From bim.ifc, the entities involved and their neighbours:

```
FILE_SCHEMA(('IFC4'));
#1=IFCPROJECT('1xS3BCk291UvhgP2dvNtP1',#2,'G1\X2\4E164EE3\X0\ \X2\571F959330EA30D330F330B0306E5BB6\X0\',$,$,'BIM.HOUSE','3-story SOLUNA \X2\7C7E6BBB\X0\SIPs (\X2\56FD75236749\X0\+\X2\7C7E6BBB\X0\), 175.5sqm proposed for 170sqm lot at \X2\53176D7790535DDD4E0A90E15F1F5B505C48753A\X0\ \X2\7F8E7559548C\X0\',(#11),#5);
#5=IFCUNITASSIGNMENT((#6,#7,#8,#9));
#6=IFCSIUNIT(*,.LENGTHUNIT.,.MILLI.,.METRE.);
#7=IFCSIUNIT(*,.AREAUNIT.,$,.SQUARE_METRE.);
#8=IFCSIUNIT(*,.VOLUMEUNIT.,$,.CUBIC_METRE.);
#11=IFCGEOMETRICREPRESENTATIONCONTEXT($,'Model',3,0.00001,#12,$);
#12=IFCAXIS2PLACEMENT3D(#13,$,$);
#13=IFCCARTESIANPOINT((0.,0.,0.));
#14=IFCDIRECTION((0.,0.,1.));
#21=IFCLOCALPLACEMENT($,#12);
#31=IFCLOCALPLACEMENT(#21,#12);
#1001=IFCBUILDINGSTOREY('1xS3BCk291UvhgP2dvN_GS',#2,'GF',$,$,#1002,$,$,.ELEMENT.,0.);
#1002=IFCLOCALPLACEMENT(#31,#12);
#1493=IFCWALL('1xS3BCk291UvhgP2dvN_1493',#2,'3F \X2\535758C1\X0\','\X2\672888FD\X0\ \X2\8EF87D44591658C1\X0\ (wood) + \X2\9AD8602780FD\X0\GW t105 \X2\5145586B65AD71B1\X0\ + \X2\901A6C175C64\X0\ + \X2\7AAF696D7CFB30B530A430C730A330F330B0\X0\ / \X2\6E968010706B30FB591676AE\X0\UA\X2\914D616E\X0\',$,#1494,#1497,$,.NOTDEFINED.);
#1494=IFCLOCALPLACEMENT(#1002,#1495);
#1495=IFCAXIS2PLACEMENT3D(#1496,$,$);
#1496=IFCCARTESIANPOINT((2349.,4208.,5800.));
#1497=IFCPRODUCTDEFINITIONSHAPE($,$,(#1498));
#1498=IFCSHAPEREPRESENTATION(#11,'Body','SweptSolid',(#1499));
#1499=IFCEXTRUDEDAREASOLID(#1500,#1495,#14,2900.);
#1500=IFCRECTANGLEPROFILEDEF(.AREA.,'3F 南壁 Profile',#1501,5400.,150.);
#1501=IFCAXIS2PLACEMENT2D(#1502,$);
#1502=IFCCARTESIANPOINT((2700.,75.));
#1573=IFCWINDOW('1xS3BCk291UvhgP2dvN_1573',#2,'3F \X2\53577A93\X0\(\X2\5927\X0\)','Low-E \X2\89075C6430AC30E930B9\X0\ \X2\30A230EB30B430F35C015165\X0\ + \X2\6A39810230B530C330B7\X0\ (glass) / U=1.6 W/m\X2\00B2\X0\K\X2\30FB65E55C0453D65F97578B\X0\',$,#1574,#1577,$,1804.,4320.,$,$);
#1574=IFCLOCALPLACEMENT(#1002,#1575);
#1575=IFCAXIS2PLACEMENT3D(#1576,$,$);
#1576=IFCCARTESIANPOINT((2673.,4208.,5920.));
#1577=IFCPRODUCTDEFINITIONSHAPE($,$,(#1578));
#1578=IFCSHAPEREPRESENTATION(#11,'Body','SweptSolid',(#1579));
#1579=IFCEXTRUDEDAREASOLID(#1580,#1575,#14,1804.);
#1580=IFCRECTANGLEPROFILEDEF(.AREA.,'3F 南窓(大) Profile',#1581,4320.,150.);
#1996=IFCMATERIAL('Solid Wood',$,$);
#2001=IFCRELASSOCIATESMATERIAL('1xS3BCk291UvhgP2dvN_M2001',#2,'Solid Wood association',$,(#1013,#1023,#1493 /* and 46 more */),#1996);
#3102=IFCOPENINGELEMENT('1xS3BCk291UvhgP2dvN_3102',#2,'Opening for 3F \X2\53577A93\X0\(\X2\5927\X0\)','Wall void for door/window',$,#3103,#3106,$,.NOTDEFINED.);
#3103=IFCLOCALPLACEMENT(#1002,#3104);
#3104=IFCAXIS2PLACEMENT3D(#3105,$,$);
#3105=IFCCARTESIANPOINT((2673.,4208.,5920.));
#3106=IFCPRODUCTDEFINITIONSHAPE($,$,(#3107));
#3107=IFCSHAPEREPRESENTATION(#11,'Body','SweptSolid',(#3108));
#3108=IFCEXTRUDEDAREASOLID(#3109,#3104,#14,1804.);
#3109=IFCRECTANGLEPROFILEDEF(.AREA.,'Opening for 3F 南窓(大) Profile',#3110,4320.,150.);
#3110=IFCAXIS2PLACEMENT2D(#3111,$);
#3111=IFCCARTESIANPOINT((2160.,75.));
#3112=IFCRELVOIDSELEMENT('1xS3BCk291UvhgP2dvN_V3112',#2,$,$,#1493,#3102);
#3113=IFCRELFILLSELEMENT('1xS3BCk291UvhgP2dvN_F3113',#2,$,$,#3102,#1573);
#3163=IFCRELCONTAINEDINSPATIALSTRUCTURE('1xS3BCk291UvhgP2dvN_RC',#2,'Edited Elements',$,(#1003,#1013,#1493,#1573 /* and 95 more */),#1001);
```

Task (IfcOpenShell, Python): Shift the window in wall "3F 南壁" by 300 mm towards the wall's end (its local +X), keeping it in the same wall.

```python
import ifcopenshell
import ifcopenshell.api.geometry
import ifcopenshell.util.placement
import ifcopenshell.util.unit

model = ifcopenshell.open("bim.ifc")
unit_scale = ifcopenshell.util.unit.calculate_unit_scale(model)

window = model.by_id(1573)
opening = window.FillsVoids[0].RelatingOpeningElement
wall = opening.VoidsElements[0].RelatingBuildingElement

wall_matrix = ifcopenshell.util.placement.get_local_placement(wall.ObjectPlacement)
shift = wall_matrix[:3, 0] * 0.3 / unit_scale
before = ifcopenshell.util.placement.get_local_placement(window.ObjectPlacement)[:3, 3].copy()

# The window is not placed relative to its opening, so move both.
for product in (opening, window):
    matrix = ifcopenshell.util.placement.get_local_placement(product.ObjectPlacement)
    matrix[:3, 3] += shift
    ifcopenshell.api.geometry.edit_object_placement(model, product=product, matrix=matrix, is_si=False)

after = ifcopenshell.util.placement.get_local_placement(window.ObjectPlacement)[:3, 3]
print("window moved by", (after - before).round(3) + 0.0)

model.write("bim_updated.ifc")
```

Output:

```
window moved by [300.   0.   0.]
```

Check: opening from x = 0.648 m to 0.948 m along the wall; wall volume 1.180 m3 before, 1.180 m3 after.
